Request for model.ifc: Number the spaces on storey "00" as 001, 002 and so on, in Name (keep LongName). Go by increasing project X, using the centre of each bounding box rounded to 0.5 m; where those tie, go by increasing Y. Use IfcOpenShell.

First a look at what the model holds.

```python
import ifcopenshell
import ifcopenshell.util.element
import ifcopenshell.util.placement

model = ifcopenshell.open("model.ifc")
print(model.schema)
storey = next(s for s in model.by_type("IfcBuildingStorey") if s.Name == "00")
spaces = [e for e in ifcopenshell.util.element.get_decomposition(storey) if e.is_a("IfcSpace")]
for e in sorted(spaces, key=lambda e: e.id()):
    origin = ifcopenshell.util.placement.get_local_placement(e.ObjectPlacement)[:3, 3]
    print(e.id(), e.Name, e.LongName, origin.round(2) + 0.0, sep=" | ")
```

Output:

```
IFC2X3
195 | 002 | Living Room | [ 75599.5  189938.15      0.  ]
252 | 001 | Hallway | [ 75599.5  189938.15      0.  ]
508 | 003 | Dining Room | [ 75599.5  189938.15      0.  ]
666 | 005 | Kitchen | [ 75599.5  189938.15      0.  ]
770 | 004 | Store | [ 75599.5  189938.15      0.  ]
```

```python
import ifcopenshell
import ifcopenshell.geom
import ifcopenshell.util.element
import ifcopenshell.util.shape

model = ifcopenshell.open("model.ifc")
settings = ifcopenshell.geom.settings()
settings.set("use-world-coords", True)


def centre(element):
    shape = ifcopenshell.geom.create_shape(settings, element)
    return ifcopenshell.util.shape.get_bbox_centroid(shape.geometry)


storey = next(s for s in model.by_type("IfcBuildingStorey") if s.Name == "00")
spaces = [e for e in ifcopenshell.util.element.get_decomposition(storey) if e.is_a("IfcSpace")]

# Insertion points can sit at a corner or the storey origin, so sort by the geometry (in metres).
centres = {e: centre(e) for e in spaces}
spaces.sort(key=lambda e: (round(centres[e][0] / 0.5), centres[e][1]))

for i, e in enumerate(spaces, start=1):
    number = f"0{i:02d}"
    e.Name = number
    print(e.id(), number)

model.write("model_updated.ifc")
```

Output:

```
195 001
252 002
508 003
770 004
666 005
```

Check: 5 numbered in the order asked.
